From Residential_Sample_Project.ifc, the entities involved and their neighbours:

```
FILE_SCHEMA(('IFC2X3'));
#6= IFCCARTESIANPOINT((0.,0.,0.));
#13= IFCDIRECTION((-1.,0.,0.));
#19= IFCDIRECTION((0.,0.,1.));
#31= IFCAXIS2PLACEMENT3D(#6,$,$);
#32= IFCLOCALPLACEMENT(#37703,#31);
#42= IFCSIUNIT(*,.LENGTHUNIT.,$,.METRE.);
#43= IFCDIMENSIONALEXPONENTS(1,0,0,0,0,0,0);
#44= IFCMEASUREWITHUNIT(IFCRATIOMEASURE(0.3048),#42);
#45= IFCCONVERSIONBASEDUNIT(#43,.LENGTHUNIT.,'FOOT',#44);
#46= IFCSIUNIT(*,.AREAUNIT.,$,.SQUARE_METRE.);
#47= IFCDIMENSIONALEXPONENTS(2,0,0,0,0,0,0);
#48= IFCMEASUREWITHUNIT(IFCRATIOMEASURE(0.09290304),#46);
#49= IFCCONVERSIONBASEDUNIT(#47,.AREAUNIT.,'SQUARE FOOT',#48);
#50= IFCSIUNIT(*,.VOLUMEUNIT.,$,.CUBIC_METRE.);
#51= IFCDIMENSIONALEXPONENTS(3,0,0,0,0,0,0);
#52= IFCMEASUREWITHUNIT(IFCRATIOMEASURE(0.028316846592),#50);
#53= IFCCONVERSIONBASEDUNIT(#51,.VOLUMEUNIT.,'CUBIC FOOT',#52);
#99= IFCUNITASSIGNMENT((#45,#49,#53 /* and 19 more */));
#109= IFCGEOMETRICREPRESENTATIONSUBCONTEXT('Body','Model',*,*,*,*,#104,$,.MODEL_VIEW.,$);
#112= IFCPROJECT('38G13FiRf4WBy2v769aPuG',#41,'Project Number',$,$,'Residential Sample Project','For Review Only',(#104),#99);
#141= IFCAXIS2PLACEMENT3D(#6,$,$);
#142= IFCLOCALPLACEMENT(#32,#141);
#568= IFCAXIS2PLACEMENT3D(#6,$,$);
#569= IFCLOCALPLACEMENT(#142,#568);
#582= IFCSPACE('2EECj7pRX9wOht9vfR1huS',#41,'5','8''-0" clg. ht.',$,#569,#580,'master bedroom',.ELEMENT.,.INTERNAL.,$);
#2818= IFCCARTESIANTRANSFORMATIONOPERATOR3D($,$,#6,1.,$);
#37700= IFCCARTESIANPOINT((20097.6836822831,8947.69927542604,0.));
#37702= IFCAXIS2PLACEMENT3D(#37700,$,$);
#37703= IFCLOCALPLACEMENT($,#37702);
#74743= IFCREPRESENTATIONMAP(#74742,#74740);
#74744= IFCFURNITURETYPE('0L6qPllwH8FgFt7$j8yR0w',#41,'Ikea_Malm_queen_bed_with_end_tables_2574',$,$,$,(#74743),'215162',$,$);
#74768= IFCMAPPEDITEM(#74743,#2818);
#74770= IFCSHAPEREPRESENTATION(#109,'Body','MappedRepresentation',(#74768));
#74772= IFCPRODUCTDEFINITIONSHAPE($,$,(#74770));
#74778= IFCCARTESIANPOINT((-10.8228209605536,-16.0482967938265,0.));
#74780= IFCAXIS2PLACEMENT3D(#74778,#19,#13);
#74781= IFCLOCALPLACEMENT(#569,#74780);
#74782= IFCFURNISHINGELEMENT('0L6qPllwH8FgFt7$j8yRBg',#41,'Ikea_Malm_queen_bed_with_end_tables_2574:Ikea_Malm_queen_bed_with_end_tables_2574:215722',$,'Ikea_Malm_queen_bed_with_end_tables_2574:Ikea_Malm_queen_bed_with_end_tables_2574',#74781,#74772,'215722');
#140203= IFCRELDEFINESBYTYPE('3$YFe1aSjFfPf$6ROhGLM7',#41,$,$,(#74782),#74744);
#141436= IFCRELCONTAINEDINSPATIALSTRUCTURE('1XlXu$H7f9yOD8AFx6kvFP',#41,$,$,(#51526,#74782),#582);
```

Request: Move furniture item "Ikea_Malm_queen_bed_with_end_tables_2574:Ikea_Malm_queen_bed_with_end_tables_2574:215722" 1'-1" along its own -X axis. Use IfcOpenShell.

```python
import ifcopenshell
import ifcopenshell.api.geometry
import ifcopenshell.util.placement
import ifcopenshell.util.unit

model = ifcopenshell.open("Residential_Sample_Project.ifc")
unit_scale = ifcopenshell.util.unit.calculate_unit_scale(model)

item = model.by_guid("0L6qPllwH8FgFt7$j8yRBg")
matrix = ifcopenshell.util.placement.get_local_placement(item.ObjectPlacement)
matrix[:3, 3] -= matrix[:3, 0] * 13 * 0.0254 / unit_scale
ifcopenshell.api.geometry.edit_object_placement(model, product=item, matrix=matrix, is_si=False)

print(ifcopenshell.util.placement.get_local_placement(item.ObjectPlacement).round(3) + 0.0)

model.write("Residential_Sample_Project_v2.ifc")
```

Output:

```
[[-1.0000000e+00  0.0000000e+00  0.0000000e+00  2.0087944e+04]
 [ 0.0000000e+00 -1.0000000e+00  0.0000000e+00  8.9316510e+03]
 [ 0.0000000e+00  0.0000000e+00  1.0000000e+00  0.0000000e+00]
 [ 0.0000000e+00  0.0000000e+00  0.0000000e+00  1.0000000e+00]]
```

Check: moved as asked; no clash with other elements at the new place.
